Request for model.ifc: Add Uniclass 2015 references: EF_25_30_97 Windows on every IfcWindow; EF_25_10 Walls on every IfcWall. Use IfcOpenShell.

First a look at what the model holds.

```python
import ifcopenshell

model = ifcopenshell.open("model.ifc")
print(model.schema)
print("classifications:", [c.Name for c in model.by_type("IfcClassification")])
for ifc_class in ("IfcDoor", "IfcRoof", "IfcStair", "IfcWall", "IfcWindow"):
    print(ifc_class, len(model.by_type(ifc_class)))
```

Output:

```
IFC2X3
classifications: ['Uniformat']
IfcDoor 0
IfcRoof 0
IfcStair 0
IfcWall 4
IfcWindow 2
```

```python
import ifcopenshell
import ifcopenshell.api.classification

model = ifcopenshell.open("model.ifc")

# IFC2X3 requires Source and Edition and has no link from the project to the system.
system = model.create_entity("IfcClassification", Source="NBS", Edition="2015", Name="Uniclass 2015")

codes = {
    "IfcWindow": ("EF_25_30_97", "Windows"),
    "IfcWall": ("EF_25_10", "Walls"),
}
for ifc_class, (code, name) in codes.items():
    products = model.by_type(ifc_class)
    ifcopenshell.api.classification.add_reference(
        model, products=products, classification=system, identification=code, name=name
    )
    print(code, len(products))

model.write("model-out.ifc")
```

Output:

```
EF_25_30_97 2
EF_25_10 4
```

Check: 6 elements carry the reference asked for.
